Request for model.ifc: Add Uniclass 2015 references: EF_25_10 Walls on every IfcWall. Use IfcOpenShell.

First a look at what the model holds.

```python
import ifcopenshell

model = ifcopenshell.open("model.ifc")
print(model.schema)
print("classifications:", [c.Name for c in model.by_type("IfcClassification")])
for ifc_class in ("IfcDoor", "IfcRoof", "IfcStair", "IfcWall", "IfcWindow"):
    print(ifc_class, len(model.by_type(ifc_class)))
```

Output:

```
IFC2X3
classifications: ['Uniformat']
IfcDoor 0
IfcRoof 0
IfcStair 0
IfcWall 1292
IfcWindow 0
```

```python
import ifcopenshell
import ifcopenshell.api.classification

model = ifcopenshell.open("model.ifc")

# IFC2X3 requires Source and Edition and has no link from the project to the system.
system = model.create_entity("IfcClassification", Source="NBS", Edition="2015", Name="Uniclass 2015")

codes = {
    "IfcWall": ("EF_25_10", "Walls"),
}
for ifc_class, (code, name) in codes.items():
    products = model.by_type(ifc_class)
    ifcopenshell.api.classification.add_reference(
        model, products=products, classification=system, identification=code, name=name
    )
    print(code, len(products))

model.write("model_updated.ifc")
```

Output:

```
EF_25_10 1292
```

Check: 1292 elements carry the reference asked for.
